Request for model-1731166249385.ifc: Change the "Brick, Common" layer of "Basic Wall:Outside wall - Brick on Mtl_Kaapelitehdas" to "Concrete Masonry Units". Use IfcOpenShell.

First a look at what the model holds.

```python
import ifcopenshell
import ifcopenshell.util.element

model = ifcopenshell.open("model-1731166249385.ifc")
print(model.schema)
for layer_set in model.by_type("IfcMaterialLayerSet"):
    if layer_set.LayerSetName == "Basic Wall:Outside wall - Brick on Mtl_Kaapelitehdas":
        for layer in layer_set.MaterialLayers:
            print(layer.id(), layer.Material and layer.Material.Name, layer.LayerThickness, sep=" | ")
        print(len(ifcopenshell.util.element.get_elements_by_material(model, layer_set)), "elements and types use it")
print(sorted(m.Name for m in model.by_type("IfcMaterial") if m.Name)[:60])
```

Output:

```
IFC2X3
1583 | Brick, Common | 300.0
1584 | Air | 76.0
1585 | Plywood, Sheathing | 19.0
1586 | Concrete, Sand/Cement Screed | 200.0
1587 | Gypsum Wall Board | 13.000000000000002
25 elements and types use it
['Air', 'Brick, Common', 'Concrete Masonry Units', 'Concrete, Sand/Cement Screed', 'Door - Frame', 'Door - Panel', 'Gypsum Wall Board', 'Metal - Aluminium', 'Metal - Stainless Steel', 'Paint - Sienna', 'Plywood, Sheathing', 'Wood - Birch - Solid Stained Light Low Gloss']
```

```python
import ifcopenshell
import ifcopenshell.api.material

model = ifcopenshell.open("model-1731166249385.ifc")

layer_set = next(s for s in model.by_type("IfcMaterialLayerSet") if s.LayerSetName == "Basic Wall:Outside wall - Brick on Mtl_Kaapelitehdas")
layer = next(l for l in layer_set.MaterialLayers if l.Material and l.Material.Name == "Brick, Common")
material = next(m for m in model.by_type("IfcMaterial") if m.Name == "Concrete Masonry Units")

# Point this one layer at the other material; renaming the old one would change it everywhere.
ifcopenshell.api.material.edit_layer(model, layer=layer, attributes={}, material=material)

print([l.Material.Name if l.Material else None for l in layer_set.MaterialLayers])

model.write("model-1731166249385_v2.ifc")
```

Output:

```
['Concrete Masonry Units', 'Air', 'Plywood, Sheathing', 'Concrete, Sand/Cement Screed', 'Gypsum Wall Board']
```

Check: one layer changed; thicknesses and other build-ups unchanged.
